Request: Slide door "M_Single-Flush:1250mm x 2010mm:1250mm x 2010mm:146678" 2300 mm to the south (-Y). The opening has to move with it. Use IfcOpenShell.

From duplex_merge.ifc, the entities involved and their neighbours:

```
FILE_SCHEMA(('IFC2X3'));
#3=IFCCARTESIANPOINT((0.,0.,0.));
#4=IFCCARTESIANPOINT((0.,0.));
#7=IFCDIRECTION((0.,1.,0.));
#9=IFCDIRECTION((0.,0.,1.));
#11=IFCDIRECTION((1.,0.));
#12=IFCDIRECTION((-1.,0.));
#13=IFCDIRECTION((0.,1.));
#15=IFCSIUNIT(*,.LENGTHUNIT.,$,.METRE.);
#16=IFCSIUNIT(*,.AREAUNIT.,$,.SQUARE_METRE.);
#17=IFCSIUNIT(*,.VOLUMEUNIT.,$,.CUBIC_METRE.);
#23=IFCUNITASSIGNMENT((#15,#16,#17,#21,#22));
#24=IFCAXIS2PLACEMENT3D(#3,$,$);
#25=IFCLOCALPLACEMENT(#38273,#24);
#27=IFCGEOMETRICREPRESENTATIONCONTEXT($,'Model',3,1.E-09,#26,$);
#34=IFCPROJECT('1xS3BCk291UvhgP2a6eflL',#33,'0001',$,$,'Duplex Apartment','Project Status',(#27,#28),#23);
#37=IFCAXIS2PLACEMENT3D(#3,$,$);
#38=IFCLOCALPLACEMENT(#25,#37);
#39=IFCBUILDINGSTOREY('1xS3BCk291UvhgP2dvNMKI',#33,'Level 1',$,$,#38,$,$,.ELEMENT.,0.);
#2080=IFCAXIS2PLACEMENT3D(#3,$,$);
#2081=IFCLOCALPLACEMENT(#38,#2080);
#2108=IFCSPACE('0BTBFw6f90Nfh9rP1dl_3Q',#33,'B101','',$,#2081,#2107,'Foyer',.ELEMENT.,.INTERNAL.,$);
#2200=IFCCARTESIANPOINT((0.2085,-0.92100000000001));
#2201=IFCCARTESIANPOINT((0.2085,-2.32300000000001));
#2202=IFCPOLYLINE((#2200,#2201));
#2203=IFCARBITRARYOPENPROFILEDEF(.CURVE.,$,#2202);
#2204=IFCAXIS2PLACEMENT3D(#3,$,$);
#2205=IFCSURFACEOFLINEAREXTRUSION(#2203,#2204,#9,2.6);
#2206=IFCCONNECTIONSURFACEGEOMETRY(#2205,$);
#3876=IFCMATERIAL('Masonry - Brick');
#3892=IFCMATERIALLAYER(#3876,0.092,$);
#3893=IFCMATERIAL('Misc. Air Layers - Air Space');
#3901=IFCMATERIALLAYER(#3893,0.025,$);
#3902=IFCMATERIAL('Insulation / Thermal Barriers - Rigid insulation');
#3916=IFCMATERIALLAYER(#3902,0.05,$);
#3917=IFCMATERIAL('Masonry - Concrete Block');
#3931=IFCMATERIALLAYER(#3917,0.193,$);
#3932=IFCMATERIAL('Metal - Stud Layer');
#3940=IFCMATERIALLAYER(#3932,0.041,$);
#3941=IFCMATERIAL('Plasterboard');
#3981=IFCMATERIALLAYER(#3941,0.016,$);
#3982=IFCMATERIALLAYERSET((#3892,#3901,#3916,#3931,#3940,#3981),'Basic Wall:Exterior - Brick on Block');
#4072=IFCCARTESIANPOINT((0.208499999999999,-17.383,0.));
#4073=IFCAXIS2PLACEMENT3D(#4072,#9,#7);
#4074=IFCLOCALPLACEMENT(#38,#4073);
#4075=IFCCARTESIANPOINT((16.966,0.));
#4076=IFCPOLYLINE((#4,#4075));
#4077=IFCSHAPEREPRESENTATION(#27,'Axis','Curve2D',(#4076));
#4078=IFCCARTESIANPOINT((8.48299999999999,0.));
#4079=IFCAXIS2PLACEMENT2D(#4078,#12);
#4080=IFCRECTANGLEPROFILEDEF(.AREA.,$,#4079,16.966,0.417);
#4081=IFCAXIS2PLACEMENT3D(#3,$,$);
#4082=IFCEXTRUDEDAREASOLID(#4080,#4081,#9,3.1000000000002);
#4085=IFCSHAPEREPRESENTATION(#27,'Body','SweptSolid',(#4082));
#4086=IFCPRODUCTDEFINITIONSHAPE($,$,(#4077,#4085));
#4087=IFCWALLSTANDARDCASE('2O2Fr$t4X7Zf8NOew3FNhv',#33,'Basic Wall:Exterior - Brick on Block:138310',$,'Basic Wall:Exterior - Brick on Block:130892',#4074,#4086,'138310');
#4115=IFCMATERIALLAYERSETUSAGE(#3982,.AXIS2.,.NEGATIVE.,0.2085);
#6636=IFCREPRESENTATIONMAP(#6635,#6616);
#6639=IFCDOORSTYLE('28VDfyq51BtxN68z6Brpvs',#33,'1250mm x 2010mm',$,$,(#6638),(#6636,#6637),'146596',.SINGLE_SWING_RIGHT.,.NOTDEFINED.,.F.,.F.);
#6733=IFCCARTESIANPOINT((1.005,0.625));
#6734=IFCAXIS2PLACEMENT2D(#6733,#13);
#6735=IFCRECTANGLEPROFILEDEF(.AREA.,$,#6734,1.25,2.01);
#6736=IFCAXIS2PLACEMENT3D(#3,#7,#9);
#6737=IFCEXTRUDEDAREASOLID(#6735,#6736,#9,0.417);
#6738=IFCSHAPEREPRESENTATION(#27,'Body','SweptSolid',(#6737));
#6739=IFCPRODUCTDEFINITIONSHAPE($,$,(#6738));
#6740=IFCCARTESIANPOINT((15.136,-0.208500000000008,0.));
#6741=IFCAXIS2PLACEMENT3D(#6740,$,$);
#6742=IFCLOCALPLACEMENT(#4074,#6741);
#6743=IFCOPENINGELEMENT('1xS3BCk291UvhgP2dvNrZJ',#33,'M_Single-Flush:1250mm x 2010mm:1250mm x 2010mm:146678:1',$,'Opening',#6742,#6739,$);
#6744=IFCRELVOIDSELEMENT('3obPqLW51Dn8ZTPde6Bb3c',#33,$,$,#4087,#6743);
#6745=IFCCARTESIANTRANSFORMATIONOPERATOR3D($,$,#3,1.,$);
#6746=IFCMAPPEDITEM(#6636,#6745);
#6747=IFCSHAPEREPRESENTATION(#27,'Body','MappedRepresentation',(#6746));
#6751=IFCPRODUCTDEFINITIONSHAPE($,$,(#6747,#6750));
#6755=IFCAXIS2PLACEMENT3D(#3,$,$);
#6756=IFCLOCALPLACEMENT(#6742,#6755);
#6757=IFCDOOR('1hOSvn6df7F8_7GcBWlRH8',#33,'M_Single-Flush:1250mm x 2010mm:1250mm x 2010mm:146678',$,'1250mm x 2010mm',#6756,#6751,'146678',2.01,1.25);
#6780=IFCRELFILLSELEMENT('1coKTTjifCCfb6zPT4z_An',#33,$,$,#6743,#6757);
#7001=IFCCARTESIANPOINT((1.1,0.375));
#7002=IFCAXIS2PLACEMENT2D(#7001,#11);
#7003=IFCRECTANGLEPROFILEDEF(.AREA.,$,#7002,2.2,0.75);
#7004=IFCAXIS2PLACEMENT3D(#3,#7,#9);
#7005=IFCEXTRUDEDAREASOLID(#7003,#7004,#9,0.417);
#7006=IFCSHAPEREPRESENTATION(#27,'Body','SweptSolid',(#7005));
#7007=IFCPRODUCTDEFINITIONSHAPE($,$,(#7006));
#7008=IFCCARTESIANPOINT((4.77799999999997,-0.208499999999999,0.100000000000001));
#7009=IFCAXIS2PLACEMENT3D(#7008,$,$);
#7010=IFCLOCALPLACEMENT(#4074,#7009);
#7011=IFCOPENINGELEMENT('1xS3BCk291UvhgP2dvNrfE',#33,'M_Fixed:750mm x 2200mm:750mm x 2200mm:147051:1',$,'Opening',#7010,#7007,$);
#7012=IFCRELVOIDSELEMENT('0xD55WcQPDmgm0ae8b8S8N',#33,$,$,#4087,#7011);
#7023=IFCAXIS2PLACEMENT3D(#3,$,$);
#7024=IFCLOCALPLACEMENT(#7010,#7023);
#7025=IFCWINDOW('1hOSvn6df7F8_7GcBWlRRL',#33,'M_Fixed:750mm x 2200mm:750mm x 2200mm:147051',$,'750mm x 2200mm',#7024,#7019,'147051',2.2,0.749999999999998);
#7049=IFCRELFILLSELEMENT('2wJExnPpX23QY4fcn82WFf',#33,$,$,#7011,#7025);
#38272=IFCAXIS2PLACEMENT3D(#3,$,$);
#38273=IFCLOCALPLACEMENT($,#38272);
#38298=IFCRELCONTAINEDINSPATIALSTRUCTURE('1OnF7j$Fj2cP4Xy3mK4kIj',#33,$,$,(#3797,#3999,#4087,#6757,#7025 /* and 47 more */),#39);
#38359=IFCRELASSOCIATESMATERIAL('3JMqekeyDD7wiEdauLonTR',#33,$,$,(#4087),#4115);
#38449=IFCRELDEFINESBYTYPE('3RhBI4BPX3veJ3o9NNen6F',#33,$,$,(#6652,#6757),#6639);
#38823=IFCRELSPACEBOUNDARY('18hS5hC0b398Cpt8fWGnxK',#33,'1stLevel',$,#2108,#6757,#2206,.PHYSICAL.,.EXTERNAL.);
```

```python
import numpy as np
import ifcopenshell
import ifcopenshell.api.geometry
import ifcopenshell.util.placement

model = ifcopenshell.open("duplex_merge.ifc")

door = model.by_guid("1hOSvn6df7F8_7GcBWlRH8")
opening = door.FillsVoids[0].RelatingOpeningElement
wall = opening.VoidsElements[0].RelatingBuildingElement

wall_matrix = ifcopenshell.util.placement.get_local_placement(wall.ObjectPlacement)
shift = wall_matrix[:3, 0] * -2.3
before = ifcopenshell.util.placement.get_local_placement(door.ObjectPlacement)[:3, 3].copy()

# The door is placed relative to its opening, so it follows when the opening moves.
matrix = ifcopenshell.util.placement.get_local_placement(opening.ObjectPlacement)
matrix[:3, 3] += shift
ifcopenshell.api.geometry.edit_object_placement(
    model, product=opening, matrix=matrix, is_si=False, should_transform_children=True
)

# Space boundary surfaces are stored in each space's coordinates; move them too.
for rel in door.ProvidesBoundaries:
    if not rel.ConnectionGeometry:
        continue
    surface = rel.ConnectionGeometry.SurfaceOnRelatingElement
    space_matrix = ifcopenshell.util.placement.get_local_placement(rel.RelatingSpace.ObjectPlacement)
    point = np.array(surface.Position.Location.Coordinates) + space_matrix[:3, :3].T @ shift
    surface.Position = model.createIfcAxis2Placement3D(
        model.createIfcCartesianPoint(point.tolist()), surface.Position.Axis, surface.Position.RefDirection
    )

after = ifcopenshell.util.placement.get_local_placement(door.ObjectPlacement)[:3, 3]
print("door moved by", (after - before).round(3) + 0.0)

model.write("duplex_merge_rev.ifc")
```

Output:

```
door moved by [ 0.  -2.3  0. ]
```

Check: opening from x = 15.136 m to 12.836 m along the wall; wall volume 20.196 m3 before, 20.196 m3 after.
